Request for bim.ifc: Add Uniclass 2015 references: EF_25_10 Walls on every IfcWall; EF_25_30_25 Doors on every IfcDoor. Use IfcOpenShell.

First a look at what the model holds.

```python
import ifcopenshell

model = ifcopenshell.open("bim.ifc")
print(model.schema)
print("classifications:", [c.Name for c in model.by_type("IfcClassification")])
for ifc_class in ("IfcDoor", "IfcRoof", "IfcStair", "IfcWall", "IfcWindow"):
    print(ifc_class, len(model.by_type(ifc_class)))
```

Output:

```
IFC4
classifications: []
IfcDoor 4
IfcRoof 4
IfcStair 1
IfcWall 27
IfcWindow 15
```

```python
import ifcopenshell
import ifcopenshell.api.classification

model = ifcopenshell.open("bim.ifc")

system = ifcopenshell.api.classification.add_classification(model, classification="Uniclass 2015")

codes = {
    "IfcWall": ("EF_25_10", "Walls"),
    "IfcDoor": ("EF_25_30_25", "Doors"),
}
for ifc_class, (code, name) in codes.items():
    products = model.by_type(ifc_class)
    ifcopenshell.api.classification.add_reference(
        model, products=products, classification=system, identification=code, name=name
    )
    print(code, len(products))

model.write("bim_edited.ifc")
```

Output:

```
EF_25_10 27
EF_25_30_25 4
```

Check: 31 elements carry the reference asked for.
